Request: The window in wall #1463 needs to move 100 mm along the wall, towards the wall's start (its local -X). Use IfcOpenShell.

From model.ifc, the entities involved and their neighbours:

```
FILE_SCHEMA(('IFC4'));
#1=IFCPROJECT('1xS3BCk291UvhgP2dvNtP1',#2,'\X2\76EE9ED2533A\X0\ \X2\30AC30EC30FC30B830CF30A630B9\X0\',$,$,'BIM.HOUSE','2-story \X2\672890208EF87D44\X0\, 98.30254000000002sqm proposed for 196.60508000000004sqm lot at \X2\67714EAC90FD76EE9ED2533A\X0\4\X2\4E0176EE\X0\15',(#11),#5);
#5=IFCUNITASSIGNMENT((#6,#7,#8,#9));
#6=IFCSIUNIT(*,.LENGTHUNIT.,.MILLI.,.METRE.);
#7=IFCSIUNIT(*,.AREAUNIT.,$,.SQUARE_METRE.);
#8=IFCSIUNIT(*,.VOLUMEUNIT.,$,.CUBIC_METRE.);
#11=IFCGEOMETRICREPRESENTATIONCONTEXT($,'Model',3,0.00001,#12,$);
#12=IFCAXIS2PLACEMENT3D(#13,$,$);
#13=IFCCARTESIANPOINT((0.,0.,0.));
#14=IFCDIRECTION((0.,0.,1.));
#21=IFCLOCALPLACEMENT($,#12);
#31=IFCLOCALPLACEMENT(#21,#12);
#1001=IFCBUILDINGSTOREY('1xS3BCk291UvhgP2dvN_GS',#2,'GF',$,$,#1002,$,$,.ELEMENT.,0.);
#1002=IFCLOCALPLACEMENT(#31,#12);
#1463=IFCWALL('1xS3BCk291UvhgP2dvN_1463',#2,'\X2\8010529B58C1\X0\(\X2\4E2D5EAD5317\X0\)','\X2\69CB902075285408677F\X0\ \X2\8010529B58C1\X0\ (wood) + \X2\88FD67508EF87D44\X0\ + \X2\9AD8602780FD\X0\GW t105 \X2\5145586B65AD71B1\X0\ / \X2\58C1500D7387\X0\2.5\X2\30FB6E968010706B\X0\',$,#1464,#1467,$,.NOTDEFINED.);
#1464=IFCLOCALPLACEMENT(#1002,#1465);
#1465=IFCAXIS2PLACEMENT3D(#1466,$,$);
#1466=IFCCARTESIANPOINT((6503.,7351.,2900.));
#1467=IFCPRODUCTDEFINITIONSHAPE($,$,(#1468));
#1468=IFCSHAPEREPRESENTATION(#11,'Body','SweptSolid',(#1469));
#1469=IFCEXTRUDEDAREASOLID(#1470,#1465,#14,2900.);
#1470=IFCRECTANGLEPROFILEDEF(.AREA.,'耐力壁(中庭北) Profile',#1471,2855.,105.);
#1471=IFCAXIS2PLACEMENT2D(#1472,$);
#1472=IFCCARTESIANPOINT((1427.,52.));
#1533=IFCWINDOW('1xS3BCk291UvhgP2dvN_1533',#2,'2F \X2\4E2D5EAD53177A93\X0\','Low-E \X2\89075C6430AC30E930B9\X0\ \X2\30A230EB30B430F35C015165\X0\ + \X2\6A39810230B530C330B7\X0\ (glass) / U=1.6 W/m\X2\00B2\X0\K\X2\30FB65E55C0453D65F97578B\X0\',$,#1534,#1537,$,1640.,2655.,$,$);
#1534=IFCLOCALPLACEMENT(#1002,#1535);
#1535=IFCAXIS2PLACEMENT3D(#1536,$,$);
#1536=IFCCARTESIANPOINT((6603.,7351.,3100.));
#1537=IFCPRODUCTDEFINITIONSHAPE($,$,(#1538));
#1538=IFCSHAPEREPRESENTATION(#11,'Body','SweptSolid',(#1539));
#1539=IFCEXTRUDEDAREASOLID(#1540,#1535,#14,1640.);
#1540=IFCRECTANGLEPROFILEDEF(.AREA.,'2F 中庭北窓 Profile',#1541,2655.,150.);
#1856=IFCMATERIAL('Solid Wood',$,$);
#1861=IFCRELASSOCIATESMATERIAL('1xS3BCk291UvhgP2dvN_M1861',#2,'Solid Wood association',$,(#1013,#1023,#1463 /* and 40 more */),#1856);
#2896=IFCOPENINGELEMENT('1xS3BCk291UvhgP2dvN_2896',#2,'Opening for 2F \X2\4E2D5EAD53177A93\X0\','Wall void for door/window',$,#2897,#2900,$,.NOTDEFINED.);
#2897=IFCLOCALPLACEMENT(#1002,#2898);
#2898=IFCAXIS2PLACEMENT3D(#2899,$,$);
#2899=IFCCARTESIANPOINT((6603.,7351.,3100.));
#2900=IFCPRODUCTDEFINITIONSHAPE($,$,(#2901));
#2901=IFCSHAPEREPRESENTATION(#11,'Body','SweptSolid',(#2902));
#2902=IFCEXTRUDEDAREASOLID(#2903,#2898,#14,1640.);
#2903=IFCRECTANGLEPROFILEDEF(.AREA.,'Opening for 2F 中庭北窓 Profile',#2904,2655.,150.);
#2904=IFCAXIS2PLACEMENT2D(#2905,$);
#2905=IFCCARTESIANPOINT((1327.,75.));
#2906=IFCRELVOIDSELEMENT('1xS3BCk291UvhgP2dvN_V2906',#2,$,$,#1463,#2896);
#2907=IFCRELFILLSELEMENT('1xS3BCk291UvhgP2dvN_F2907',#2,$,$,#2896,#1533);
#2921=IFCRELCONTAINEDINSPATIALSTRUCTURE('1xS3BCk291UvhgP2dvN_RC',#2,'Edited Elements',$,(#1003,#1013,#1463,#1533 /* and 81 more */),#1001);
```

```python
import ifcopenshell
import ifcopenshell.api.geometry
import ifcopenshell.util.placement
import ifcopenshell.util.unit

model = ifcopenshell.open("model.ifc")
unit_scale = ifcopenshell.util.unit.calculate_unit_scale(model)

window = model.by_id(1533)
opening = window.FillsVoids[0].RelatingOpeningElement
wall = opening.VoidsElements[0].RelatingBuildingElement

wall_matrix = ifcopenshell.util.placement.get_local_placement(wall.ObjectPlacement)
shift = wall_matrix[:3, 0] * -0.1 / unit_scale
before = ifcopenshell.util.placement.get_local_placement(window.ObjectPlacement)[:3, 3].copy()

# The window is not placed relative to its opening, so move both.
for product in (opening, window):
    matrix = ifcopenshell.util.placement.get_local_placement(product.ObjectPlacement)
    matrix[:3, 3] += shift
    ifcopenshell.api.geometry.edit_object_placement(model, product=product, matrix=matrix, is_si=False)

after = ifcopenshell.util.placement.get_local_placement(window.ObjectPlacement)[:3, 3]
print("window moved by", (after - before).round(3) + 0.0)

model.write("model_v2.ifc")
```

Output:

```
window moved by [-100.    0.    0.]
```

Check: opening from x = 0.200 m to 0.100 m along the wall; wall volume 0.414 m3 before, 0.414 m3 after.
